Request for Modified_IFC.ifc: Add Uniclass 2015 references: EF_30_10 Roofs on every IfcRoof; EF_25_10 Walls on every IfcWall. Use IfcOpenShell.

First a look at what the model holds.

```python
import ifcopenshell

model = ifcopenshell.open("Modified_IFC.ifc")
print(model.schema)
print("classifications:", [c.Name for c in model.by_type("IfcClassification")])
for ifc_class in ("IfcDoor", "IfcRoof", "IfcStair", "IfcWall", "IfcWindow"):
    print(ifc_class, len(model.by_type(ifc_class)))
```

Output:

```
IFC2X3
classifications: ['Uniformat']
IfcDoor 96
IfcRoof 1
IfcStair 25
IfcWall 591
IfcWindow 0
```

```python
import ifcopenshell
import ifcopenshell.api.classification

model = ifcopenshell.open("Modified_IFC.ifc")

# IFC2X3 requires Source and Edition and has no link from the project to the system.
system = model.create_entity("IfcClassification", Source="NBS", Edition="2015", Name="Uniclass 2015")

codes = {
    "IfcRoof": ("EF_30_10", "Roofs"),
    "IfcWall": ("EF_25_10", "Walls"),
}
for ifc_class, (code, name) in codes.items():
    products = model.by_type(ifc_class)
    ifcopenshell.api.classification.add_reference(
        model, products=products, classification=system, identification=code, name=name
    )
    print(code, len(products))

model.write("Modified_IFC_v2.ifc")
```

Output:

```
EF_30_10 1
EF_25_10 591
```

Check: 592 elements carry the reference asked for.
